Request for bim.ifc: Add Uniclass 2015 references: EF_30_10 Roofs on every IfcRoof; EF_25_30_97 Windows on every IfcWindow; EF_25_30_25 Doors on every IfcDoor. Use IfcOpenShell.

First a look at what the model holds.

```python
import ifcopenshell

model = ifcopenshell.open("bim.ifc")
print(model.schema)
print("classifications:", [c.Name for c in model.by_type("IfcClassification")])
for ifc_class in ("IfcDoor", "IfcRoof", "IfcStair", "IfcWall", "IfcWindow"):
    print(ifc_class, len(model.by_type(ifc_class)))
```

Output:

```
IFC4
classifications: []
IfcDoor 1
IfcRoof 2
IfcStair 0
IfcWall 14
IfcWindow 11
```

```python
import ifcopenshell
import ifcopenshell.api.classification

model = ifcopenshell.open("bim.ifc")

system = ifcopenshell.api.classification.add_classification(model, classification="Uniclass 2015")

codes = {
    "IfcRoof": ("EF_30_10", "Roofs"),
    "IfcWindow": ("EF_25_30_97", "Windows"),
    "IfcDoor": ("EF_25_30_25", "Doors"),
}
for ifc_class, (code, name) in codes.items():
    products = model.by_type(ifc_class)
    ifcopenshell.api.classification.add_reference(
        model, products=products, classification=system, identification=code, name=name
    )
    print(code, len(products))

model.write("bim-out.ifc")
```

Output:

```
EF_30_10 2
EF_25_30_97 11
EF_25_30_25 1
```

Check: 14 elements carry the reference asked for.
